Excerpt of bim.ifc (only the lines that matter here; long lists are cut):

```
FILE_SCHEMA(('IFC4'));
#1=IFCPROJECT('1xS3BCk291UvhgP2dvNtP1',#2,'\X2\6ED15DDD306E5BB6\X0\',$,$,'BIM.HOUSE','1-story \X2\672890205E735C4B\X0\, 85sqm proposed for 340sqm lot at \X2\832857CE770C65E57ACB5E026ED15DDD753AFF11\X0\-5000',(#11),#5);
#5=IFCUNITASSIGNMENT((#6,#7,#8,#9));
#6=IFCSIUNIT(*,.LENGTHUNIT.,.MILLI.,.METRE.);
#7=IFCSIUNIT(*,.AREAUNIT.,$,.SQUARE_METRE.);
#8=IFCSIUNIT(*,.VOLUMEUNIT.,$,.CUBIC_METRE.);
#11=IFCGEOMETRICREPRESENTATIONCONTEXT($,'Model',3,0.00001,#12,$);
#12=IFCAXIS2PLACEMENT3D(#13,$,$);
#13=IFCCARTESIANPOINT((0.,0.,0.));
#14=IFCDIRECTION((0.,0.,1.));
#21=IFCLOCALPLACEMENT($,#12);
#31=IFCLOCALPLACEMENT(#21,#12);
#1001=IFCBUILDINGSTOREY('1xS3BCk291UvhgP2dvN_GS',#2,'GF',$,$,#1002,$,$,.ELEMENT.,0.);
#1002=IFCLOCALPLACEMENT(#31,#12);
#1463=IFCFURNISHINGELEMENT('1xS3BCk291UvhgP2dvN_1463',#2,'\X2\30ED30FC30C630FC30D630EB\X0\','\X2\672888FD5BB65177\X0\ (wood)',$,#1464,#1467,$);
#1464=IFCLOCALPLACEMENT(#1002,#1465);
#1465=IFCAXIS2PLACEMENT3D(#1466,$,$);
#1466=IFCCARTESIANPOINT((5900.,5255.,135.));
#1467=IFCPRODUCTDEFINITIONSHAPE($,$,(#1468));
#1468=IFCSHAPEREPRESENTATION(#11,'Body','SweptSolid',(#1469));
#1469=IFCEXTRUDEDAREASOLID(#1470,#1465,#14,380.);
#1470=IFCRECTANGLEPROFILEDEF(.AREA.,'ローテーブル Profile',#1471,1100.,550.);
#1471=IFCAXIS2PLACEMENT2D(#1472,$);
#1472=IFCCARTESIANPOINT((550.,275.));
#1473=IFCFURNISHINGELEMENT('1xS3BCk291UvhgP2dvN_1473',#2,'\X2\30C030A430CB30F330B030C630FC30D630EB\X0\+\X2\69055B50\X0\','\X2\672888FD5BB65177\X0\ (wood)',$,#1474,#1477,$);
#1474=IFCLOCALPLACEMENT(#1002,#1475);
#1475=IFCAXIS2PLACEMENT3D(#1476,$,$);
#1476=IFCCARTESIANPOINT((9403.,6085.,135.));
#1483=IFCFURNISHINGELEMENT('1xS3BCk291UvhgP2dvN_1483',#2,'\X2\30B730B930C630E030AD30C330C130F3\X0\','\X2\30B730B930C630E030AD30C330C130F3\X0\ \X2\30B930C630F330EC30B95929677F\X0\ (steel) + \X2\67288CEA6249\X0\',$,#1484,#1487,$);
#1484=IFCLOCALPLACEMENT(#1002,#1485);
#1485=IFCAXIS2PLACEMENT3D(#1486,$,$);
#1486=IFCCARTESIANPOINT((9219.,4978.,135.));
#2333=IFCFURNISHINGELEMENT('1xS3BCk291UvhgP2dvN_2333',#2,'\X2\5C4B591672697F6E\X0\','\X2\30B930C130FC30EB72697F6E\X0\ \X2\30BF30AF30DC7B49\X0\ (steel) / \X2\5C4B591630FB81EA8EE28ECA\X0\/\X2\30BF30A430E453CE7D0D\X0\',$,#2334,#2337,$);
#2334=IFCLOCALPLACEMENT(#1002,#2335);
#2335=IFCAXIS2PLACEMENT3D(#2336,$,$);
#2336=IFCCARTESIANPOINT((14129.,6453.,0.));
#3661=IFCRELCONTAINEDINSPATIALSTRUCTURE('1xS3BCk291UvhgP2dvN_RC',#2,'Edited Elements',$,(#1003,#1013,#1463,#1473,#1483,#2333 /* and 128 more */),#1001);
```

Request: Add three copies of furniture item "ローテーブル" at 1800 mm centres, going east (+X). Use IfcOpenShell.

```python
import numpy as np
import ifcopenshell
import ifcopenshell.api.geometry
import ifcopenshell.api.root
import ifcopenshell.util.element
import ifcopenshell.util.placement

model = ifcopenshell.open("bim.ifc")


def reuse_history(source, copy):
    """copy_class also copies each property set's owner history, people and application; keep the originals."""
    for rel in copy.IsDefinedBy:
        if rel.is_a("IfcRelDefinesByProperties") and (history := rel.RelatingPropertyDefinition.OwnerHistory):
            rel.RelatingPropertyDefinition.OwnerHistory = source.OwnerHistory
            ifcopenshell.util.element.remove_deep2(model, history)


source = model.by_guid("1xS3BCk291UvhgP2dvN_1463")
base = ifcopenshell.util.placement.get_local_placement(source.ObjectPlacement)
step = np.array([1.0, 0.0, 0.0]) * 1800.0

for i in range(1, 4):
    copy = ifcopenshell.api.root.copy_class(model, product=source)
    copy.Representation = ifcopenshell.util.element.copy_deep(
        model, source.Representation, exclude=["IfcGeometricRepresentationContext", "IfcRepresentationMap"]
    )
    reuse_history(source, copy)
    matrix = base.copy()
    matrix[:3, 3] += i * step
    print("added at", matrix[:3, 3].round(3) + 0.0)
    ifcopenshell.api.geometry.edit_object_placement(model, product=copy, matrix=matrix, is_si=False)

model.write("bim-out.ifc")
```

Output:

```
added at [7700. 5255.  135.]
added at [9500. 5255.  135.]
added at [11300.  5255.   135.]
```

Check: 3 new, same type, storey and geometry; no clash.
